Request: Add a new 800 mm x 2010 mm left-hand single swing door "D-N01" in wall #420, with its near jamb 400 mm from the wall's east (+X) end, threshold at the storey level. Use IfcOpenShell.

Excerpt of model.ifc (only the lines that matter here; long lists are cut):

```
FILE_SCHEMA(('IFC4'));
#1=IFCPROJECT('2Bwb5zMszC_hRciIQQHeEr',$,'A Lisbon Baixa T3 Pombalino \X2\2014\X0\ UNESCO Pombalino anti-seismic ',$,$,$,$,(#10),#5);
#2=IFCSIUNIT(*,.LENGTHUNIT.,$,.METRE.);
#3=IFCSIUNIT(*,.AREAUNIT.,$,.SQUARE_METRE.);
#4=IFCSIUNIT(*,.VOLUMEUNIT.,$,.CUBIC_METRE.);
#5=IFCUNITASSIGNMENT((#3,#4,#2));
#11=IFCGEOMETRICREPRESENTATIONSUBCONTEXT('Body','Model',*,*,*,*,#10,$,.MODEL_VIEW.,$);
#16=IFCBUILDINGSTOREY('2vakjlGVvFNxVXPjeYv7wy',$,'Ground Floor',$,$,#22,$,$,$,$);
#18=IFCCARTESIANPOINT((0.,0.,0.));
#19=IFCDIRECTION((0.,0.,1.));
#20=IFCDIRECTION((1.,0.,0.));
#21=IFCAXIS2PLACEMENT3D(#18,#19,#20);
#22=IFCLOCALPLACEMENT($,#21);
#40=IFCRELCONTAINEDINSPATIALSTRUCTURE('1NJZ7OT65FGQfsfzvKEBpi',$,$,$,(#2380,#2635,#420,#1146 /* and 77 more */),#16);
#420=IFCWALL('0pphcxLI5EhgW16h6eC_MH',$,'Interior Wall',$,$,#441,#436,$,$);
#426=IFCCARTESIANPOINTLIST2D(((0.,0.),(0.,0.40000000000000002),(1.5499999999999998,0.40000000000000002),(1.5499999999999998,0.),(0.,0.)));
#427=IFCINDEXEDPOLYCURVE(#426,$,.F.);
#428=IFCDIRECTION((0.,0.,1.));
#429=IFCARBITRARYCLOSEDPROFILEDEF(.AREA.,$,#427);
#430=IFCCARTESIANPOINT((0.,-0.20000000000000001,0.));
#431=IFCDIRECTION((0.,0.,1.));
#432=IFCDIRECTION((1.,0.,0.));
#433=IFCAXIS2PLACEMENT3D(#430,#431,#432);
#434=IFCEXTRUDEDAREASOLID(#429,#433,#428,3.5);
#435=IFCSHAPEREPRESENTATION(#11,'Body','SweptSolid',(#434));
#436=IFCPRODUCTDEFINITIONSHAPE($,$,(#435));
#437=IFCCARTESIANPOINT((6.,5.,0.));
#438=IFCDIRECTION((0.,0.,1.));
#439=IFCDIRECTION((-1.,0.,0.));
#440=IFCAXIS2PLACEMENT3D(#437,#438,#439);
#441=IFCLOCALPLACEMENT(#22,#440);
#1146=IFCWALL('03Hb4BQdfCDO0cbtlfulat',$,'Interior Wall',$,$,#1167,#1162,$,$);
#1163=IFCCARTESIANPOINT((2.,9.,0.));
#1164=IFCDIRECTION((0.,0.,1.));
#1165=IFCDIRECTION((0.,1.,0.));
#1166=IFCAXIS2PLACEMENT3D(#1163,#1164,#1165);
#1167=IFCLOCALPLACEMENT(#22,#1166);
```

```python
import numpy as np
import ifcopenshell
import ifcopenshell.api.feature
import ifcopenshell.api.geometry
import ifcopenshell.api.root
import ifcopenshell.api.spatial
import ifcopenshell.geom
import ifcopenshell.util.element
import ifcopenshell.util.placement
import ifcopenshell.util.representation
import ifcopenshell.util.shape
import ifcopenshell.util.unit

model = ifcopenshell.open("model.ifc")
unit_scale = ifcopenshell.util.unit.calculate_unit_scale(model)
settings = ifcopenshell.geom.settings()


def volume(element):
    """Net volume in cubic metres, openings subtracted."""
    shape = ifcopenshell.geom.create_shape(settings, element)
    return ifcopenshell.util.shape.get_volume(shape.geometry)


wall = model.by_guid("0pphcxLI5EhgW16h6eC_MH")
storey = ifcopenshell.util.element.get_container(wall, ifc_class="IfcBuildingStorey")
context = ifcopenshell.util.representation.get_context(model, "Model", "Body", "MODEL_VIEW")
before = volume(wall)

width, height, from_end, sill = 0.8, 2.01, 0.4, 0.0  # metres

# The wall runs along its own X axis, and the end named is its -X end.
wall_shape = ifcopenshell.geom.create_shape(settings, wall)
x, y, z = ifcopenshell.util.shape.get_vertices(wall_shape.geometry).T
start = x.min() + from_end
face, thickness = float(y.min()), float(y.max() - y.min())
wall_matrix = ifcopenshell.util.placement.get_local_placement(wall.ObjectPlacement)
level = ifcopenshell.util.placement.get_local_placement(storey.ObjectPlacement)[2, 3]


def in_wall(x, y):
    """Placement at x, y metres in the wall's axes, at sill height."""
    matrix = wall_matrix.copy()
    matrix[:, 3] = wall_matrix @ np.array([x / unit_scale, y / unit_scale, 0.0, 1.0])
    matrix[2, 3] = level + sill / unit_scale
    return matrix


# Opening: a box that overshoots both wall faces by 50 mm.
opening = ifcopenshell.api.root.create_entity(model, ifc_class="IfcOpeningElement", predefined_type="OPENING")
box = ifcopenshell.api.geometry.add_wall_representation(
    model, context=context, length=width, height=height, thickness=thickness + 0.1
)
ifcopenshell.api.geometry.assign_representation(model, product=opening, representation=box)
ifcopenshell.api.geometry.edit_object_placement(model, product=opening, matrix=in_wall(start, face - 0.05), is_si=False)
ifcopenshell.api.feature.add_feature(model, feature=opening, element=wall)

door = ifcopenshell.api.root.create_entity(model, ifc_class="IfcDoor", name="D-N01", predefined_type="DOOR")
door.OverallWidth, door.OverallHeight = width / unit_scale, height / unit_scale
door.OperationType = "SINGLE_SWING_LEFT"
body = ifcopenshell.api.geometry.add_door_representation(
    model,
    context=context,
    overall_width=door.OverallWidth,
    overall_height=door.OverallHeight,
    operation_type="SINGLE_SWING_LEFT",
    lining_properties={"LiningDepth": thickness / unit_scale, "ThresholdDepth": thickness / unit_scale},
)
ifcopenshell.api.geometry.assign_representation(model, product=door, representation=body)
ifcopenshell.api.spatial.assign_container(model, products=[door], relating_structure=storey)
ifcopenshell.api.feature.add_filling(model, opening=opening, element=door)

# The lining spans the wall, so the door starts at the wall face.
ifcopenshell.api.geometry.edit_object_placement(model, product=door, matrix=in_wall(start, face), is_si=False)

after = volume(wall)

print(f"wall volume {before:.3f} -> {after:.3f} m3")

model.write("model_updated.ifc")
```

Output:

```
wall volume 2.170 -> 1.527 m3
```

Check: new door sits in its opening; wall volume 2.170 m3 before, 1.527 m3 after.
